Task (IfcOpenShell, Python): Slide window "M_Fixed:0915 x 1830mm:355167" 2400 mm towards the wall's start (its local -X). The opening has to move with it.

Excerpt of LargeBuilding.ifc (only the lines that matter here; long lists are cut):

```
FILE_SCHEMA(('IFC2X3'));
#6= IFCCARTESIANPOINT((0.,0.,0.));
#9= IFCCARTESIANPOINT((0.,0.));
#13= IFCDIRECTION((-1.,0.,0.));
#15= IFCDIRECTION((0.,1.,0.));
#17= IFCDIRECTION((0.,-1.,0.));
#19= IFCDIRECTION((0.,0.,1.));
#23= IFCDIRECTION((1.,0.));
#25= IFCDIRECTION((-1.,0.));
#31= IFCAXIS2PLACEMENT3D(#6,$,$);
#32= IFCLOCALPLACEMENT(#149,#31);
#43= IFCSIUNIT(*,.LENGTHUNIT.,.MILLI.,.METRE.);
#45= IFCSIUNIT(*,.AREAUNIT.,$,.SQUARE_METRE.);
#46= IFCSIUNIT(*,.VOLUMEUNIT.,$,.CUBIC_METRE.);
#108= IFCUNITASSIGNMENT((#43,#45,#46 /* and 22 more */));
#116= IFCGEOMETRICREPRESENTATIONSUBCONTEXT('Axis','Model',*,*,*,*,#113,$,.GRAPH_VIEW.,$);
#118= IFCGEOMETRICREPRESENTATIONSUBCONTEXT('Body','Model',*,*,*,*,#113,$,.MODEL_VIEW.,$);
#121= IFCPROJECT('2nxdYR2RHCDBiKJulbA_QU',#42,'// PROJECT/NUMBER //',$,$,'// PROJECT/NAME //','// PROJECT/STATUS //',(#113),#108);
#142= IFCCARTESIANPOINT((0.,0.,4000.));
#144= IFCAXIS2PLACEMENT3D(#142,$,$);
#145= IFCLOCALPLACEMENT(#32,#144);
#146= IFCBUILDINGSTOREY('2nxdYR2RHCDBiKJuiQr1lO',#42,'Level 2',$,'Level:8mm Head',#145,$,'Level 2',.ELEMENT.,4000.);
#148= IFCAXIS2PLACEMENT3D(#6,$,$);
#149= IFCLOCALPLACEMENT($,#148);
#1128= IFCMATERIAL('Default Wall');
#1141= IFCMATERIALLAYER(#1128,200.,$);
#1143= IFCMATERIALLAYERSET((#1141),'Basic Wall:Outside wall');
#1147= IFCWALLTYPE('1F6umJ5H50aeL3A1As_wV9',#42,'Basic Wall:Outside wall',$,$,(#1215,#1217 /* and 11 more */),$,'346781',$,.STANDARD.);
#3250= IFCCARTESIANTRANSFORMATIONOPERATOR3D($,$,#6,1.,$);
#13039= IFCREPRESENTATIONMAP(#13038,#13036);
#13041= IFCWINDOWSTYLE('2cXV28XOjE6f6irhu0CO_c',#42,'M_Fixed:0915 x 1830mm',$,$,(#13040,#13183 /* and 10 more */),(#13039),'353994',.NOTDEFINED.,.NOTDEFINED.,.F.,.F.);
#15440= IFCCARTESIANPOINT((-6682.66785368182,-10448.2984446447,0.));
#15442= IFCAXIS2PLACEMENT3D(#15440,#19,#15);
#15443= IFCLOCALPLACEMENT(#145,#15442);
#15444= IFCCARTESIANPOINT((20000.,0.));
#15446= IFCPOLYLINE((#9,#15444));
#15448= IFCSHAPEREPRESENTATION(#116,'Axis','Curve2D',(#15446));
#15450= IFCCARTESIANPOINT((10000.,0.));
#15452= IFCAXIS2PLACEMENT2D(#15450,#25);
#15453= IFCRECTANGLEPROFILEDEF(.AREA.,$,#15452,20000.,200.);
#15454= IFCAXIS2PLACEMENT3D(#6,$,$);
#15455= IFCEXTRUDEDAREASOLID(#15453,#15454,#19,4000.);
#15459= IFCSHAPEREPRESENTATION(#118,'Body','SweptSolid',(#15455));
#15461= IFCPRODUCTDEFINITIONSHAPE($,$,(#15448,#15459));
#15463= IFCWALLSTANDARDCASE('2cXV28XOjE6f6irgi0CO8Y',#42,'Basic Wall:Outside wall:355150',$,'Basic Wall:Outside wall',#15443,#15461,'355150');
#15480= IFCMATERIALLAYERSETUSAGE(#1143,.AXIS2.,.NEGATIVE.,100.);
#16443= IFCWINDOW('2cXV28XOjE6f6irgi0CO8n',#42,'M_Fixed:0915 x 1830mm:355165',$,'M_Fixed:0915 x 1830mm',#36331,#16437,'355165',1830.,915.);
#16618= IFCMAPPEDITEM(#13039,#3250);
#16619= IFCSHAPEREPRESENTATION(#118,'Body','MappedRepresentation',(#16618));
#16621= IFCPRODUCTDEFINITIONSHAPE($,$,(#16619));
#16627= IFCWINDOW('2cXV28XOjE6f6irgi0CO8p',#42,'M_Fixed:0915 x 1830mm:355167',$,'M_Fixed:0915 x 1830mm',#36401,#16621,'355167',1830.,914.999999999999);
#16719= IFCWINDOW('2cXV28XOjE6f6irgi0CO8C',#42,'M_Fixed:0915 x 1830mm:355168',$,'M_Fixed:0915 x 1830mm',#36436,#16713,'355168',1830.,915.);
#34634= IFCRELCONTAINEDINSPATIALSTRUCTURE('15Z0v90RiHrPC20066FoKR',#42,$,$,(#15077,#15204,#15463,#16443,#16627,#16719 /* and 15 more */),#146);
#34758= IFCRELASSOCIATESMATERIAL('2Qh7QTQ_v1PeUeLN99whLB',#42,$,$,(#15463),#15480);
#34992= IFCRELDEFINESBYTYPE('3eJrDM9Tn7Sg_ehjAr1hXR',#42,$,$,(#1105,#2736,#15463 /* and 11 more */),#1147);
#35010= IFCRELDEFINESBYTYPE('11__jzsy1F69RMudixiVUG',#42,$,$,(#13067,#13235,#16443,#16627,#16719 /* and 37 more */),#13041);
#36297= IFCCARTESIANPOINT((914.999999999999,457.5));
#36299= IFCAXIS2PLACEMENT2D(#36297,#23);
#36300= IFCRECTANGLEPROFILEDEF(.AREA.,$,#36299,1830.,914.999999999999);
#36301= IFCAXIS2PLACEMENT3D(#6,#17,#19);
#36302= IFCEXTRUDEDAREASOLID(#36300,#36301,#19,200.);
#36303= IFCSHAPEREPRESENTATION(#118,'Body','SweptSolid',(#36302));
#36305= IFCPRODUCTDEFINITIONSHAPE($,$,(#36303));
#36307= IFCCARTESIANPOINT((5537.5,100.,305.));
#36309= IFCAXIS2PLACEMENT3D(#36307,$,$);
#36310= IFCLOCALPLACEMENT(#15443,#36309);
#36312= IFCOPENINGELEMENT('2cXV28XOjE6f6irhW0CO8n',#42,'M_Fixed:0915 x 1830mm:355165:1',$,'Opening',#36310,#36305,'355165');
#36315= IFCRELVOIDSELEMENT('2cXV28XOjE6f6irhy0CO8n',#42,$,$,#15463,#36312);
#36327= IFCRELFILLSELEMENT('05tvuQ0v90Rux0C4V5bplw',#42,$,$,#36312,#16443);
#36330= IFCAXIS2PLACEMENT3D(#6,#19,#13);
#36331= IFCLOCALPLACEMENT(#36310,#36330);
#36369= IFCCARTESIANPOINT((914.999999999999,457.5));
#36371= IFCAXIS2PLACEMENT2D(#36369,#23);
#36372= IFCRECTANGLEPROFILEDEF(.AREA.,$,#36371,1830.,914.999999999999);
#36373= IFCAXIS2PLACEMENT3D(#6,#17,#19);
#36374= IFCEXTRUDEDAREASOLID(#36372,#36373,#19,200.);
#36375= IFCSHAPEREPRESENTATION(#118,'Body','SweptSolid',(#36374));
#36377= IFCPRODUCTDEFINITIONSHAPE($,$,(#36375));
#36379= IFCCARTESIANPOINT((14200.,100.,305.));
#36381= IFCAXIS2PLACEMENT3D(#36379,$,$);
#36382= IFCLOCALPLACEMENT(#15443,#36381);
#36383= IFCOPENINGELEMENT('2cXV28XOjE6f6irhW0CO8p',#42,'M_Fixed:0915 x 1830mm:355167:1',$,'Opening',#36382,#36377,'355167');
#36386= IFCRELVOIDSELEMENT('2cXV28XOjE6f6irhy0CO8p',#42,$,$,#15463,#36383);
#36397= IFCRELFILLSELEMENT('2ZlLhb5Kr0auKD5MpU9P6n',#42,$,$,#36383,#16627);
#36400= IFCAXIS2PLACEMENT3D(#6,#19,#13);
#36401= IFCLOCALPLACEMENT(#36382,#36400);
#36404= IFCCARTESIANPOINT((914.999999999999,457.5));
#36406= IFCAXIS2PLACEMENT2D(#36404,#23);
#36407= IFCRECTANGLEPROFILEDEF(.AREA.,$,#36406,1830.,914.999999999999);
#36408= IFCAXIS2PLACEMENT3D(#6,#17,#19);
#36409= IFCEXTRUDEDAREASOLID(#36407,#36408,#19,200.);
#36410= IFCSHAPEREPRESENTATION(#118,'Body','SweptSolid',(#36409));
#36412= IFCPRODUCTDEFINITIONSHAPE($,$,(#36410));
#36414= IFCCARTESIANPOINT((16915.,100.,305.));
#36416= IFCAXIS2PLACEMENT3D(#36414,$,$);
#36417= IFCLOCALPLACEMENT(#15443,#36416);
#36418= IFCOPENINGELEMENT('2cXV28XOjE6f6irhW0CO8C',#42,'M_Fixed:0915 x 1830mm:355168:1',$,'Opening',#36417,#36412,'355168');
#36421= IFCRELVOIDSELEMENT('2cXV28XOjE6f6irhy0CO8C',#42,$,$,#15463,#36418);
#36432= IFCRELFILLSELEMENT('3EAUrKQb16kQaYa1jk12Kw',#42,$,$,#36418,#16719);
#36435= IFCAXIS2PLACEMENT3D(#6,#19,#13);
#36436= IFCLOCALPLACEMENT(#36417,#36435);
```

```python
import ifcopenshell
import ifcopenshell.api.geometry
import ifcopenshell.util.placement

model = ifcopenshell.open("LargeBuilding.ifc")

window = model.by_guid("2cXV28XOjE6f6irgi0CO8p")
opening = window.FillsVoids[0].RelatingOpeningElement
wall = opening.VoidsElements[0].RelatingBuildingElement

wall_matrix = ifcopenshell.util.placement.get_local_placement(wall.ObjectPlacement)
shift = wall_matrix[:3, 0] * -2400.0
before = ifcopenshell.util.placement.get_local_placement(window.ObjectPlacement)[:3, 3].copy()

# The window is placed relative to its opening, so it follows when the opening moves.
matrix = ifcopenshell.util.placement.get_local_placement(opening.ObjectPlacement)
matrix[:3, 3] += shift
ifcopenshell.api.geometry.edit_object_placement(
    model, product=opening, matrix=matrix, is_si=False, should_transform_children=True
)

after = ifcopenshell.util.placement.get_local_placement(window.ObjectPlacement)[:3, 3]
print("window moved by", (after - before).round(3) + 0.0)

model.write("LargeBuilding_v2.ifc")
```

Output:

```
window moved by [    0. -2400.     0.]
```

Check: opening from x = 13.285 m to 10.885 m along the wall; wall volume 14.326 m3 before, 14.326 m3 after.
